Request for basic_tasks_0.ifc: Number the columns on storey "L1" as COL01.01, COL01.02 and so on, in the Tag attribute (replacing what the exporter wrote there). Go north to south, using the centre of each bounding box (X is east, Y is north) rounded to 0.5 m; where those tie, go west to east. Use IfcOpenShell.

First a look at what the model holds.

```python
import ifcopenshell
import ifcopenshell.util.element
import ifcopenshell.util.placement

model = ifcopenshell.open("basic_tasks_0.ifc")
print(model.schema)
storey = next(s for s in model.by_type("IfcBuildingStorey") if s.Name == "L1")
columns = [e for e in ifcopenshell.util.element.get_decomposition(storey) if e.is_a("IfcColumn")]
for e in sorted(columns, key=lambda e: e.id()):
    origin = ifcopenshell.util.placement.get_local_placement(e.ObjectPlacement)[:3, 3]
    print(e.id(), e.Tag, e.Name, origin.round(2) + 0.0, sep=" | ")
```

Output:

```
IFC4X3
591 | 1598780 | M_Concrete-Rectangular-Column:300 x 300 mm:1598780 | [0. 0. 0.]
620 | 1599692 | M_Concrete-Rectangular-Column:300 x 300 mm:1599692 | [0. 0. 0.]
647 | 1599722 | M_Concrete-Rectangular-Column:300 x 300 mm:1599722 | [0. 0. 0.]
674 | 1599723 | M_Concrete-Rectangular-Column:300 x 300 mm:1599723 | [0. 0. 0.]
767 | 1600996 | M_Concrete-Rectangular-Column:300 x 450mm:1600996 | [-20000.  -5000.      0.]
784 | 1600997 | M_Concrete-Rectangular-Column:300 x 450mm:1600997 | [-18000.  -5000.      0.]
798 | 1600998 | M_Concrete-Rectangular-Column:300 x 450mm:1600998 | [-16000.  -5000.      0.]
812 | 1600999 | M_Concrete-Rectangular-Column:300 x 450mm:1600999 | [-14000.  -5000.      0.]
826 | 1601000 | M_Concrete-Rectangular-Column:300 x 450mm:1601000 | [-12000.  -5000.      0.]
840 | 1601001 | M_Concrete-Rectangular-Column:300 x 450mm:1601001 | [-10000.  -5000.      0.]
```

```python
import ifcopenshell
import ifcopenshell.geom
import ifcopenshell.util.element
import ifcopenshell.util.shape

model = ifcopenshell.open("basic_tasks_0.ifc")
settings = ifcopenshell.geom.settings()
settings.set("use-world-coords", True)


def centre(element):
    shape = ifcopenshell.geom.create_shape(settings, element)
    return ifcopenshell.util.shape.get_bbox_centroid(shape.geometry)


storey = next(s for s in model.by_type("IfcBuildingStorey") if s.Name == "L1")
columns = [e for e in ifcopenshell.util.element.get_decomposition(storey) if e.is_a("IfcColumn")]

# Insertion points can sit at a corner or the storey origin, so sort by the geometry (in metres).
centres = {e: centre(e) for e in columns}
columns.sort(key=lambda e: (-round(centres[e][1] / 0.5), centres[e][0]))

for i, e in enumerate(columns, start=1):
    number = f"COL01.{i:02d}"
    e.Tag = number
    print(e.id(), number)

model.write("basic_tasks_0_v2.ifc")
```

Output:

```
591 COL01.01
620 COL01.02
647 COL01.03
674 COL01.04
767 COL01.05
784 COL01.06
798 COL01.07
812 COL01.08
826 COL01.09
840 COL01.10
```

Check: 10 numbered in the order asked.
